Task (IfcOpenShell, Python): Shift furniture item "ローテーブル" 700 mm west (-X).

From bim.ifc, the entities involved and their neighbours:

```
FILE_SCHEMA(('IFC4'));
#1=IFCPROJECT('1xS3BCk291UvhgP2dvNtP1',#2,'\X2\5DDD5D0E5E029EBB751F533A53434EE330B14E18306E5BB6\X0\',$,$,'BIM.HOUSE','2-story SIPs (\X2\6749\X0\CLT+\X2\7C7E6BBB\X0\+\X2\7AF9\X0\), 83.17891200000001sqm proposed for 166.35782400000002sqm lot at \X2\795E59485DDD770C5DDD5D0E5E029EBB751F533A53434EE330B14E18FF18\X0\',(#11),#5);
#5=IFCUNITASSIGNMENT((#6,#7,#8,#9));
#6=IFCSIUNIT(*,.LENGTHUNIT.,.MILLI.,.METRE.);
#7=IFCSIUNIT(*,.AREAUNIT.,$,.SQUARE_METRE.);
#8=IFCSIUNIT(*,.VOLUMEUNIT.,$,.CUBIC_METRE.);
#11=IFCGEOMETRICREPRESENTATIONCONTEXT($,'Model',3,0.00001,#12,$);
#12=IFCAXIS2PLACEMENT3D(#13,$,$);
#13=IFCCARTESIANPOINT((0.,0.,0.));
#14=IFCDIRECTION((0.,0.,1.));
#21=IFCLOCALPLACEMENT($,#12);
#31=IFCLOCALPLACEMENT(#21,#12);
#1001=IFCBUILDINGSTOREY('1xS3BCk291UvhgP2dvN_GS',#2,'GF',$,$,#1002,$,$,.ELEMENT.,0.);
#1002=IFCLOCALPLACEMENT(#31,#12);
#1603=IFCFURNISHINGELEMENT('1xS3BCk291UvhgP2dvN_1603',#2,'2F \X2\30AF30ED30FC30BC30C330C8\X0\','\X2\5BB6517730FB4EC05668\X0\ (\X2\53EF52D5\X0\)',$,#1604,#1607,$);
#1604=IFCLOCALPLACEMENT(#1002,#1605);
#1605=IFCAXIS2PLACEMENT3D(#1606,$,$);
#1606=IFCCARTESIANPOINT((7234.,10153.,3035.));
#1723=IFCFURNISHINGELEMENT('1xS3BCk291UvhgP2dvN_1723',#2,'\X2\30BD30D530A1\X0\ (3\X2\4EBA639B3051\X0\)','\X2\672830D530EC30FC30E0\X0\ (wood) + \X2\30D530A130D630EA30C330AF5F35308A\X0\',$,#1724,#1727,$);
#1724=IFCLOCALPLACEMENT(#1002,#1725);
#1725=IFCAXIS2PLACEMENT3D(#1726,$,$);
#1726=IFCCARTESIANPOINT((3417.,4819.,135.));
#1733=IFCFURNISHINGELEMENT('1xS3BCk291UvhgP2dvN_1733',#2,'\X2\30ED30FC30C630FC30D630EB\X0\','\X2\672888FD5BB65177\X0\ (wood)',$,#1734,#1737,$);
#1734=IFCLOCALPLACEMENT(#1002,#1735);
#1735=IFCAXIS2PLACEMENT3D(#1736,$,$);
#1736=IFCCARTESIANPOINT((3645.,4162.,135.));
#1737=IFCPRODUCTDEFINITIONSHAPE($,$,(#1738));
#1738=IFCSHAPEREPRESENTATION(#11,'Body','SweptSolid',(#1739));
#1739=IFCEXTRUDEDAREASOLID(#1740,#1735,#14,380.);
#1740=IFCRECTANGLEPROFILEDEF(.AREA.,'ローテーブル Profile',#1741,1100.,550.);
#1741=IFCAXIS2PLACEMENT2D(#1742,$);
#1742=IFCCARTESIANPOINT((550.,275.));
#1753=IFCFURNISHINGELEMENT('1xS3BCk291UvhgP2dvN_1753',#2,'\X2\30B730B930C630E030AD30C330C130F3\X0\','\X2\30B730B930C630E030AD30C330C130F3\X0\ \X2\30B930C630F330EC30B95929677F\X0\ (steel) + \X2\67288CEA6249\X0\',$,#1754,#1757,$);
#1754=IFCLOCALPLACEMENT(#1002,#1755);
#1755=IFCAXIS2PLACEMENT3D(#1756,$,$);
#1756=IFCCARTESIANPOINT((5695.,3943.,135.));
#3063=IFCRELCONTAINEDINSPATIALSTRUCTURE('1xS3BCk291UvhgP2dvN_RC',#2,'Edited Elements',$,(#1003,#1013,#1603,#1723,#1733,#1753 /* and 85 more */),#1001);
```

```python
import ifcopenshell
import ifcopenshell.api.geometry
import ifcopenshell.util.placement
import ifcopenshell.util.unit

model = ifcopenshell.open("bim.ifc")
unit_scale = ifcopenshell.util.unit.calculate_unit_scale(model)

item = model.by_id(1733)
matrix = ifcopenshell.util.placement.get_local_placement(item.ObjectPlacement)
matrix[0, 3] -= 0.7 / unit_scale
ifcopenshell.api.geometry.edit_object_placement(model, product=item, matrix=matrix, is_si=False)

print(ifcopenshell.util.placement.get_local_placement(item.ObjectPlacement).round(3) + 0.0)

model.write("bim-out.ifc")
```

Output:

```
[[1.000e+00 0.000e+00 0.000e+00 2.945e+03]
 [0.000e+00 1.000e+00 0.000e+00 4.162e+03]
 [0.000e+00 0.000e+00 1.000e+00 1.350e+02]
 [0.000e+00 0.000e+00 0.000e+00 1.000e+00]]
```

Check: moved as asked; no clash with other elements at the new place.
